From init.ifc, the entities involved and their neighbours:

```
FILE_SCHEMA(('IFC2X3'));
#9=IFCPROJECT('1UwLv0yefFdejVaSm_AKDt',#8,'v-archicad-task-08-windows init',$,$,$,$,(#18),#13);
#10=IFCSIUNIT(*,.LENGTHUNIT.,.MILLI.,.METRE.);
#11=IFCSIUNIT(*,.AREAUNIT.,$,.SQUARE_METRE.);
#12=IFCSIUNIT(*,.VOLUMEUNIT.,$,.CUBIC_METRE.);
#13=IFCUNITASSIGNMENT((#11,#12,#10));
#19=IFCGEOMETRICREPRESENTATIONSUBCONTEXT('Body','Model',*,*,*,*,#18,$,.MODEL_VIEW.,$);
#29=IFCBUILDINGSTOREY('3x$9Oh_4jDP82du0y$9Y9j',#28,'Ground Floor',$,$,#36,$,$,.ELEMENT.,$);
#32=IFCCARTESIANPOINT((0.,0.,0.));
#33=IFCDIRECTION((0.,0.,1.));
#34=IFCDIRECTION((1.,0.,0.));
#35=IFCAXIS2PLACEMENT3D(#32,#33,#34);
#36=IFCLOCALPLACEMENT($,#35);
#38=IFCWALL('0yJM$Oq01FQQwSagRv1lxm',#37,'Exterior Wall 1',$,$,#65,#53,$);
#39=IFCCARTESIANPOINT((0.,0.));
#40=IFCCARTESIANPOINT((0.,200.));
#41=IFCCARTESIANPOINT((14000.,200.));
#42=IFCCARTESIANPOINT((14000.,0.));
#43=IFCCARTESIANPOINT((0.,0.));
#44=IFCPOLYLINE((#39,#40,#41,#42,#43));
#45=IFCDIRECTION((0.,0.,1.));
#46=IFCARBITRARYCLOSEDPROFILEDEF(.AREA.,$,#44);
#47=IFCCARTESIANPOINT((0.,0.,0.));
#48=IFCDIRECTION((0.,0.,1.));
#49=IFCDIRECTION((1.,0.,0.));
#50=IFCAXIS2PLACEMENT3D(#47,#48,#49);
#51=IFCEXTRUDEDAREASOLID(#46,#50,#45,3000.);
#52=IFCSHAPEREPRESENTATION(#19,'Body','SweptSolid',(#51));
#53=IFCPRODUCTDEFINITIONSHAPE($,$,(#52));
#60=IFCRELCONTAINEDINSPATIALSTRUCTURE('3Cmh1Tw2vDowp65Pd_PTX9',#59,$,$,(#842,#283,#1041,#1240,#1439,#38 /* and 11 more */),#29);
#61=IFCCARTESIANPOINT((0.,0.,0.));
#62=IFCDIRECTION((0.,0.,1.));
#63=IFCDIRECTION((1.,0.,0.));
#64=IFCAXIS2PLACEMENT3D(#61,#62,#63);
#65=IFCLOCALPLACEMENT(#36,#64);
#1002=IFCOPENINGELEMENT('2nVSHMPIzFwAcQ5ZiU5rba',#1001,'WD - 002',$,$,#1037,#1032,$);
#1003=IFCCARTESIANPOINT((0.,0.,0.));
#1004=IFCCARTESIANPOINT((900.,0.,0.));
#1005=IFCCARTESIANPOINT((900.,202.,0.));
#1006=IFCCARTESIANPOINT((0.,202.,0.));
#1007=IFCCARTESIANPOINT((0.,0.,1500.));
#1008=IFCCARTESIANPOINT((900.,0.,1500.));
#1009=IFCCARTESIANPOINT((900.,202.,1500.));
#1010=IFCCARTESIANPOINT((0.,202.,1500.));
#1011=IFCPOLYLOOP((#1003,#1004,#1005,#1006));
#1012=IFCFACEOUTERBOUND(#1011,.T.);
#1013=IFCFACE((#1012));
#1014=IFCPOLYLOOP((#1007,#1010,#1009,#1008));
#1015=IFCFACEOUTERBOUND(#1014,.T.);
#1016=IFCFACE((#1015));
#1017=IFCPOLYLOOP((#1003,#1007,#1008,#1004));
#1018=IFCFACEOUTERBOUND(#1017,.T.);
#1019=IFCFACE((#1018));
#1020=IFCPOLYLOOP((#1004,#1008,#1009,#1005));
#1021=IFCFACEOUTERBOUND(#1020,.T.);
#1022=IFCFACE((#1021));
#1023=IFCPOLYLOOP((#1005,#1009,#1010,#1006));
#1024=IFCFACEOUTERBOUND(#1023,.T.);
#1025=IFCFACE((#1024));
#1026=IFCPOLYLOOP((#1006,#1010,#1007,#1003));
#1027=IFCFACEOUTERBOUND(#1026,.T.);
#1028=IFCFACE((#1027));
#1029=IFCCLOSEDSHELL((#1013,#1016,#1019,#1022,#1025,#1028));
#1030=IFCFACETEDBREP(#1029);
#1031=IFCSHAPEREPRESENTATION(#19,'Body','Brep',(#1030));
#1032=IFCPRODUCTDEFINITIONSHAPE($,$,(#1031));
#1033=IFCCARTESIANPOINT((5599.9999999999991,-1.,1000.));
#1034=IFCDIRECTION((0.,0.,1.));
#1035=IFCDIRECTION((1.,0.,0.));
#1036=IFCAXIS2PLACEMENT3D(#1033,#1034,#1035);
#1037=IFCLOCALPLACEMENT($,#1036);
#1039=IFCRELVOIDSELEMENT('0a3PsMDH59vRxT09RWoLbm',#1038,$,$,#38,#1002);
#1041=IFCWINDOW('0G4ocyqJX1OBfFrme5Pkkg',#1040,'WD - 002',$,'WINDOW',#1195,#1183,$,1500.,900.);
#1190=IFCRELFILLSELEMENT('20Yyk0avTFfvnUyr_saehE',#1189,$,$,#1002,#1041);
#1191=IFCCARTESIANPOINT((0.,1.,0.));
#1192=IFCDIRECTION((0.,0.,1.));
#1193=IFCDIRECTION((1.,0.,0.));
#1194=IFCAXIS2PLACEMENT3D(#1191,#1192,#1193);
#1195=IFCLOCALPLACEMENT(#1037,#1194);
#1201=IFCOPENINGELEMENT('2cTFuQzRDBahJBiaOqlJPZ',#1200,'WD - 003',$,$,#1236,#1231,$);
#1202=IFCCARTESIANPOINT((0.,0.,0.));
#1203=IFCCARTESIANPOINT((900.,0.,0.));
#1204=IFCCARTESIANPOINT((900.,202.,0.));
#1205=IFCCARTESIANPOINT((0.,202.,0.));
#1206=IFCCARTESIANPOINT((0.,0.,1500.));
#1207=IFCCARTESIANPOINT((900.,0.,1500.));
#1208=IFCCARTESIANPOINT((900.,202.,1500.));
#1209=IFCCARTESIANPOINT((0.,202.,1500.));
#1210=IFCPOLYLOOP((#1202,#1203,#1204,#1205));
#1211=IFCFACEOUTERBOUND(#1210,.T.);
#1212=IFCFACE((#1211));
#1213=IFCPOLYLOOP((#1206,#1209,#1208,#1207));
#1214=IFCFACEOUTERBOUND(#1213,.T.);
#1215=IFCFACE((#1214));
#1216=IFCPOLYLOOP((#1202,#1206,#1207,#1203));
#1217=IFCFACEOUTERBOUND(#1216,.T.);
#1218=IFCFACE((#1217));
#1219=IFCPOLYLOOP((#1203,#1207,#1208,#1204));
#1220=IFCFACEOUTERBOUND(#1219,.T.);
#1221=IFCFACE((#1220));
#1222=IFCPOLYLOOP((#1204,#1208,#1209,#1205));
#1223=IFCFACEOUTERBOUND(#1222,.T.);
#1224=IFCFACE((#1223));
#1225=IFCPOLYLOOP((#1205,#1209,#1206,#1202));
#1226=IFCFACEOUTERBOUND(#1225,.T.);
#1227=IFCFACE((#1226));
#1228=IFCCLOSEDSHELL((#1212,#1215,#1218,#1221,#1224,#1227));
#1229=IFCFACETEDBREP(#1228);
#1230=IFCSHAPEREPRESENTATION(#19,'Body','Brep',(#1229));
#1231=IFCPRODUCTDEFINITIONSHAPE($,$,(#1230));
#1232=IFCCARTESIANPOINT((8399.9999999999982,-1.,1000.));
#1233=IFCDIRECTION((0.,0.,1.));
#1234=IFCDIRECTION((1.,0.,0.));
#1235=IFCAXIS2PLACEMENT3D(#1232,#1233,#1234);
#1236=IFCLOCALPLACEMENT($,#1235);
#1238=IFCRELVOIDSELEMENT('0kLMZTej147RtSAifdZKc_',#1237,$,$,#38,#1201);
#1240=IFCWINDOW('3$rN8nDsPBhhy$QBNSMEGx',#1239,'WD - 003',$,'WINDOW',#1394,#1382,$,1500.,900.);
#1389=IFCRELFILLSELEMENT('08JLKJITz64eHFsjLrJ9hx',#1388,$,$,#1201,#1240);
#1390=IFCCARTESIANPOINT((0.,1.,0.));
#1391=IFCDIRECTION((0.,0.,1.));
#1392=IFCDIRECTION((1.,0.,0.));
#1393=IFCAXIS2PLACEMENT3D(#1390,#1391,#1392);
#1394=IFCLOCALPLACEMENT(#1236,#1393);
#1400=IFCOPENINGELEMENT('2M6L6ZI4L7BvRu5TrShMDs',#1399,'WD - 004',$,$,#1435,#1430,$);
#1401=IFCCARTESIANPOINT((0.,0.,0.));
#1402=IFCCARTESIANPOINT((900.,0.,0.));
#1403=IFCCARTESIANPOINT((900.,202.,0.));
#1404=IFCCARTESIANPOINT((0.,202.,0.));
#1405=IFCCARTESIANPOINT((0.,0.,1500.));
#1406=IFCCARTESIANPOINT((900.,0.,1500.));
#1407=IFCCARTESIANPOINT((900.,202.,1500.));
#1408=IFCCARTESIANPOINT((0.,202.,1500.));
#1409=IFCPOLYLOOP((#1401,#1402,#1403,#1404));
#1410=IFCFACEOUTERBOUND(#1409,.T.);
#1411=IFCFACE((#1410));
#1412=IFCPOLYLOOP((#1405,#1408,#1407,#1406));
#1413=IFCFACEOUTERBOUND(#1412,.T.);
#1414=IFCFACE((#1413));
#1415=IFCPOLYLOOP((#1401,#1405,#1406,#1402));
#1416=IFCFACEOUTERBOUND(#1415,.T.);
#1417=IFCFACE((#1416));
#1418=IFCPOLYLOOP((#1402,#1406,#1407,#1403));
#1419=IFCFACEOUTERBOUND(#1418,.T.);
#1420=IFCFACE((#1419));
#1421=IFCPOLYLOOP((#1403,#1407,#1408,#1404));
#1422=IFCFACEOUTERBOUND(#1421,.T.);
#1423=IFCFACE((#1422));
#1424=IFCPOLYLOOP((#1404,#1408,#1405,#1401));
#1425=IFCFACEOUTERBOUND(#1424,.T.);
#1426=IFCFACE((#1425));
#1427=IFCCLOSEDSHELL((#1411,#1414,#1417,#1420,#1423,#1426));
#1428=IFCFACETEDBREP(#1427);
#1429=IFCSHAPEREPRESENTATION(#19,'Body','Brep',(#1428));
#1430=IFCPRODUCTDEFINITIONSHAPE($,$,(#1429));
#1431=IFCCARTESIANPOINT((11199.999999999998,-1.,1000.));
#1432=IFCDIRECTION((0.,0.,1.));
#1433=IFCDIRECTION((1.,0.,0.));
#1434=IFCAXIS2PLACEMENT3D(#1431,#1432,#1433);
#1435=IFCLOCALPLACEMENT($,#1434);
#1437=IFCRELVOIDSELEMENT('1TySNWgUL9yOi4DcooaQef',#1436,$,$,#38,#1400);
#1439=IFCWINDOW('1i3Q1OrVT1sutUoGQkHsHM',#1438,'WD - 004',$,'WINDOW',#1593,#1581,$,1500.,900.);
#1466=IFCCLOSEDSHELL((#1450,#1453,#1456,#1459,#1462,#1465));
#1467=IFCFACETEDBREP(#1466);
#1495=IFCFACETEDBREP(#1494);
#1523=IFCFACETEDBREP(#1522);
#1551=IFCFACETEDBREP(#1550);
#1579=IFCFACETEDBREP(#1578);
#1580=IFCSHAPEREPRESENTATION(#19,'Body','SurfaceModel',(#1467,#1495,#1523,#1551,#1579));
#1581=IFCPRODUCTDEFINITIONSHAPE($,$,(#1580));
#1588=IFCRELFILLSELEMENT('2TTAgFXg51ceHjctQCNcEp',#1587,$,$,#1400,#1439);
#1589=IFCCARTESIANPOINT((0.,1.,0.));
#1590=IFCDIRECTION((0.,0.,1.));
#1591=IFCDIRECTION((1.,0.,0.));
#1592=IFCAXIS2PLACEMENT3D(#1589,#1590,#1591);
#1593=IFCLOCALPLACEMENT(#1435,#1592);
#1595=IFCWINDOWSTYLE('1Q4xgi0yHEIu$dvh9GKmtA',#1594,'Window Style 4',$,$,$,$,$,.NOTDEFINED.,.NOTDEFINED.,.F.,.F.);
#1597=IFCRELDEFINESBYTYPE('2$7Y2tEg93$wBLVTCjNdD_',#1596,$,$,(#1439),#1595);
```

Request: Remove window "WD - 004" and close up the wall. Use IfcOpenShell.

```python
import ifcopenshell
import ifcopenshell.api.feature
import ifcopenshell.api.root
import ifcopenshell.geom
import ifcopenshell.util.shape

model = ifcopenshell.open("init.ifc")
settings = ifcopenshell.geom.settings()


def volume(element):
    """Net volume in cubic metres, openings subtracted."""
    shape = ifcopenshell.geom.create_shape(settings, element)
    return ifcopenshell.util.shape.get_volume(shape.geometry)


window = model.by_guid("1i3Q1OrVT1sutUoGQkHsHM")
opening = window.FillsVoids[0].RelatingOpeningElement
wall = opening.VoidsElements[0].RelatingBuildingElement
before = volume(wall)

ifcopenshell.api.root.remove_product(model, product=window)
ifcopenshell.api.feature.remove_feature(model, feature=opening)

after = volume(wall)

print(f"wall volume {before:.3f} -> {after:.3f} m3")

model.write("init_v2.ifc")
```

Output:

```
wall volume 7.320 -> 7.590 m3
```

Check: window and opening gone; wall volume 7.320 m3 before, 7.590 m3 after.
